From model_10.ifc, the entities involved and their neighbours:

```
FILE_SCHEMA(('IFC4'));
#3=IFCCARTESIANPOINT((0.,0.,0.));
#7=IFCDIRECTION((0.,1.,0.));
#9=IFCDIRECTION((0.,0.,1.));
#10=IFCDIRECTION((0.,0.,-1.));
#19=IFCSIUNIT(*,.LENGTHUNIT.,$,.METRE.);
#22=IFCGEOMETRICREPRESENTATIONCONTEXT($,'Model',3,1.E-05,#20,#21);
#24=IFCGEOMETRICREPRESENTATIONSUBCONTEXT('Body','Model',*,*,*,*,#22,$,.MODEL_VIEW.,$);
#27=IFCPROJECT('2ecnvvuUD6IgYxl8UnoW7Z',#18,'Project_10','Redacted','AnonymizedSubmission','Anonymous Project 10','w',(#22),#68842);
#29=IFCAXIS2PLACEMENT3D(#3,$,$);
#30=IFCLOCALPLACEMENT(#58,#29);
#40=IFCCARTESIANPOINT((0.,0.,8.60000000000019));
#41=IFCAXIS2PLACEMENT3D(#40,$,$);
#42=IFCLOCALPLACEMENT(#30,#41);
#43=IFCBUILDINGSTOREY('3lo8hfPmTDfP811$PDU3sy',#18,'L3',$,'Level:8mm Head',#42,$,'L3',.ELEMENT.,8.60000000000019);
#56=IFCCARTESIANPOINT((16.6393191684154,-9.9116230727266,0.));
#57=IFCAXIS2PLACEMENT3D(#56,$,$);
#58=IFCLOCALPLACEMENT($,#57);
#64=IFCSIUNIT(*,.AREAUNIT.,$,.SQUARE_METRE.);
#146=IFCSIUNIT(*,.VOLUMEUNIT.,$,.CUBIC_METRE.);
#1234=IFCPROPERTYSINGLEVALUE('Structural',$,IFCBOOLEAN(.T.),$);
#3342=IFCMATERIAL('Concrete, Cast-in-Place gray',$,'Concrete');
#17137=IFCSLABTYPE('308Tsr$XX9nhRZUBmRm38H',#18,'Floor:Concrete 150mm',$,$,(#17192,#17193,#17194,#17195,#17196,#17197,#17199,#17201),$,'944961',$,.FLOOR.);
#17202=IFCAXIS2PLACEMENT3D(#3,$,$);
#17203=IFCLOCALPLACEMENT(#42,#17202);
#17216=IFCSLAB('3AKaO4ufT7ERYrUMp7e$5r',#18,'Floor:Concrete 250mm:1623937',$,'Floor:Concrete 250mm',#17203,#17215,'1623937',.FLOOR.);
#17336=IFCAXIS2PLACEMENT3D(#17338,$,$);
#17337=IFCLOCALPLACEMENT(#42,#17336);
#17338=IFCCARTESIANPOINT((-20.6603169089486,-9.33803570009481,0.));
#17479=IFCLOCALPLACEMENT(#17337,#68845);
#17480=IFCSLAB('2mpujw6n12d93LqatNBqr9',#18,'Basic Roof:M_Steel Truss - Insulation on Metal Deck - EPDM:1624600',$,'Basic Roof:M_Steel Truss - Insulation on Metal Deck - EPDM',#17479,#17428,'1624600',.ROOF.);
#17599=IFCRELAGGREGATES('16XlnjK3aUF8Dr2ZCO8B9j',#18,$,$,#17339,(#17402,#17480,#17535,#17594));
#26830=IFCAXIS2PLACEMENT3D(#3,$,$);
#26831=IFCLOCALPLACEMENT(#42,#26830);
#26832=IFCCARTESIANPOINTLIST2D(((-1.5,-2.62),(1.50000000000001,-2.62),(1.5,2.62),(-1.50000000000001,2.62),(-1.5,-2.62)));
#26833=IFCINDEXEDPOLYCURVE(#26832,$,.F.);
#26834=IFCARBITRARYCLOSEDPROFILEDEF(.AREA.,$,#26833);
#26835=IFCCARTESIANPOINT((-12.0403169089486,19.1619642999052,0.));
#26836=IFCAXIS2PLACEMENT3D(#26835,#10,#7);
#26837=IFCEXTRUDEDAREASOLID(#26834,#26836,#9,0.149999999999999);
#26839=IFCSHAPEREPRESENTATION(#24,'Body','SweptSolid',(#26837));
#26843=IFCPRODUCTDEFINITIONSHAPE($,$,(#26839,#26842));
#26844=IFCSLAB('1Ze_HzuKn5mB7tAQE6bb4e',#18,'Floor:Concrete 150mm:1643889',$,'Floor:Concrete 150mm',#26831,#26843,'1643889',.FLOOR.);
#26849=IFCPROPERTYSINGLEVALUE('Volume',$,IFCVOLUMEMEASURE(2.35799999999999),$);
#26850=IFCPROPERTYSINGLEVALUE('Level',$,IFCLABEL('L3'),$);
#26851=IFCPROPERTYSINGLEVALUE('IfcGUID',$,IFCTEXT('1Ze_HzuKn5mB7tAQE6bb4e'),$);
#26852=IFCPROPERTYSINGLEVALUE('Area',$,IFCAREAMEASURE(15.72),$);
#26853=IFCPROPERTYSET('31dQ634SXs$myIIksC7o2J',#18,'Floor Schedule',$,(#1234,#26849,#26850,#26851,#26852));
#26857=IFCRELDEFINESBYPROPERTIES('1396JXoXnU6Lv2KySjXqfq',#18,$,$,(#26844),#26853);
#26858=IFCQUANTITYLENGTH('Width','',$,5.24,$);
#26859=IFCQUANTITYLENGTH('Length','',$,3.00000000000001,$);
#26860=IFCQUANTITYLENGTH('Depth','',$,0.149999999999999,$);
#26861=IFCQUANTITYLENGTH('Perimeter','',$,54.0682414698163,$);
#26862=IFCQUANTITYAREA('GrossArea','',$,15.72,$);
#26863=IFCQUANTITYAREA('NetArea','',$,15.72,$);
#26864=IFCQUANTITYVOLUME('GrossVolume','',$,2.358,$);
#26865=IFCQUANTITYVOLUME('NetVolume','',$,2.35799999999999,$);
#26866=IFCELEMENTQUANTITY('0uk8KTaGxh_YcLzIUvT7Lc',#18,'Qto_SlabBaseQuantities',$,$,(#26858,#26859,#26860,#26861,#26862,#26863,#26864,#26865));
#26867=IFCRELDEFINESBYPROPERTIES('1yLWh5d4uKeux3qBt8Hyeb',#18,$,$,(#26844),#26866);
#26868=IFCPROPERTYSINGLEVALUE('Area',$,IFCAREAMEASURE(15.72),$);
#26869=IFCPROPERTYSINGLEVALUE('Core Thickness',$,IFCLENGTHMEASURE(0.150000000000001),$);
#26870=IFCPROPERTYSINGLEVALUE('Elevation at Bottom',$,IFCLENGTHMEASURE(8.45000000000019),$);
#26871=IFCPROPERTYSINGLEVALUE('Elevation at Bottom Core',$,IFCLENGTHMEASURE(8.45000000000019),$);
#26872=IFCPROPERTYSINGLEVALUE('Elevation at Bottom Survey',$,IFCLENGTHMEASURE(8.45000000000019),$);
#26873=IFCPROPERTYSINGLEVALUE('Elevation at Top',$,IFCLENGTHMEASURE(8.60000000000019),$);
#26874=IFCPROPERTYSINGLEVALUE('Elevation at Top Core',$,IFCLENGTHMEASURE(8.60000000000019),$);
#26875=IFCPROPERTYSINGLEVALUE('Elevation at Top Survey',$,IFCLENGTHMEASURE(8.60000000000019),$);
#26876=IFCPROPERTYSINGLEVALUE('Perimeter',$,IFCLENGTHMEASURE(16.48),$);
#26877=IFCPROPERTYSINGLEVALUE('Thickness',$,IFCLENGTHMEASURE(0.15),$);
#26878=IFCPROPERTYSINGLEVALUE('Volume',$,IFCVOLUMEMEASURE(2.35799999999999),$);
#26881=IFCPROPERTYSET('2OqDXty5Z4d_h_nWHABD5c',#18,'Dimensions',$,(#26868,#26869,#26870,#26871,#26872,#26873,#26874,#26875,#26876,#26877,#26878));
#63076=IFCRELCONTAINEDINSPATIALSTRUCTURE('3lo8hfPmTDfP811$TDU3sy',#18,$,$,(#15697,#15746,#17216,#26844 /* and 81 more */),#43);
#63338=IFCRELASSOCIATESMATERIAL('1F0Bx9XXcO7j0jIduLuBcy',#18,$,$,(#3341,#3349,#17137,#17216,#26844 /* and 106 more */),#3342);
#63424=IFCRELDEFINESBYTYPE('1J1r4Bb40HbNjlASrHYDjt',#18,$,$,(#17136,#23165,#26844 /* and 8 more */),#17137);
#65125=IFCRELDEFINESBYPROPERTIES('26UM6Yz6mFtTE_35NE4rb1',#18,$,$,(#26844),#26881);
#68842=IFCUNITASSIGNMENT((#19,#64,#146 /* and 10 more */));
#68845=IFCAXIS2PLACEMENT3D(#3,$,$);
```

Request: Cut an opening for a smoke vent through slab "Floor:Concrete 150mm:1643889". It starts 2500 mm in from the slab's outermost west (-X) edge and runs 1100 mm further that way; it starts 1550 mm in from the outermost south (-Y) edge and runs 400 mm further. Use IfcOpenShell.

```python
import numpy as np
import ifcopenshell
import ifcopenshell.api.feature
import ifcopenshell.api.geometry
import ifcopenshell.api.pset
import ifcopenshell.api.root
import ifcopenshell.geom
import ifcopenshell.util.element
import ifcopenshell.util.placement
import ifcopenshell.util.representation
import ifcopenshell.util.shape
import ifcopenshell.util.unit

model = ifcopenshell.open("model_10.ifc")
unit_scale = ifcopenshell.util.unit.calculate_unit_scale(model)
area_scale = ifcopenshell.util.unit.calculate_unit_scale(model, "AREAUNIT")
volume_scale = ifcopenshell.util.unit.calculate_unit_scale(model, "VOLUMEUNIT")
settings = ifcopenshell.geom.settings()


def volume(element):
    """Net volume in cubic metres, openings subtracted."""
    shape = ifcopenshell.geom.create_shape(settings, element)
    return ifcopenshell.util.shape.get_volume(shape.geometry)


slab = model.by_guid("1Ze_HzuKn5mB7tAQE6bb4e")
before = volume(slab)

# Extent in the slab's own axes, in metres. The edges named are its -X and -Y sides.
slab_shape = ifcopenshell.geom.create_shape(settings, slab)
vertices = ifcopenshell.util.shape.get_vertices(slab_shape.geometry)
x_min, y_min, bottom = vertices.min(axis=0)
top = vertices[:, 2].max()

opening = ifcopenshell.api.root.create_entity(model, ifc_class="IfcOpeningElement", name="Smoke vent opening", predefined_type="OPENING")
context = ifcopenshell.util.representation.get_context(model, "Model", "Body", "MODEL_VIEW")
width, depth = 1.1, 0.4
outline = [(0.0, 0.0), (width, 0.0), (width, depth), (0.0, depth), (0.0, 0.0)]
# Overshoot both faces by 50 mm so the cut is clean.
shape = ifcopenshell.api.geometry.add_slab_representation(
    model, context=context, depth=top - bottom + 0.1, polyline=outline
)
ifcopenshell.api.geometry.assign_representation(model, product=opening, representation=shape)

matrix = ifcopenshell.util.placement.get_local_placement(slab.ObjectPlacement)
matrix[:, 3] = matrix @ np.append(np.array([x_min + 2.5, y_min + 1.55, bottom - 0.05]) / unit_scale, 1.0)
ifcopenshell.api.geometry.edit_object_placement(model, product=opening, matrix=matrix, is_si=False)
ifcopenshell.api.feature.add_feature(model, feature=opening, element=slab)

after = volume(slab)

# Update the slab's stored quantities.
pset = model.by_id(ifcopenshell.util.element.get_pset(slab, "Floor Schedule", should_inherit=False)["id"])
ifcopenshell.api.pset.edit_pset(model, pset=pset, properties={
    "Volume": model.create_entity("IfcVolumeMeasure", after / volume_scale),
    "Area": model.create_entity("IfcAreaMeasure", after / (top - bottom) / area_scale),
})
qto = model.by_id(ifcopenshell.util.element.get_pset(slab, "Qto_SlabBaseQuantities", should_inherit=False)["id"])
ifcopenshell.api.pset.edit_qto(model, qto=qto, properties={
    "NetArea": after / (top - bottom) / area_scale,
    "NetVolume": after / volume_scale,
})
pset = model.by_id(ifcopenshell.util.element.get_pset(slab, "Dimensions", should_inherit=False)["id"])
ifcopenshell.api.pset.edit_pset(model, pset=pset, properties={
    "Area": model.create_entity("IfcAreaMeasure", after / (top - bottom) / area_scale),
    "Volume": model.create_entity("IfcVolumeMeasure", after / volume_scale),
})

print(f"slab volume {before:.3f} -> {after:.3f} m3")

model.write("model_10_v2.ifc")
```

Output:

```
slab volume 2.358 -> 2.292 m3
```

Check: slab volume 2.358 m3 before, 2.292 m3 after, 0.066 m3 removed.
